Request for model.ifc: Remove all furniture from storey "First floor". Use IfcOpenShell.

First a look at what the model holds.

```python
import ifcopenshell
import ifcopenshell.util.element

model = ifcopenshell.open("model.ifc")
print(model.schema)
storey = next(s for s in model.by_type("IfcBuildingStorey") if s.Name == "First floor")
furniture = [e for e in ifcopenshell.util.element.get_decomposition(storey) if e.is_a("IfcFurnishingElement")]
seen = {}
for e in furniture:
    element_type = ifcopenshell.util.element.get_type(e)
    name = element_type.Name if element_type not in (None, e) else None
    seen[name] = seen.get(name, 0) + 1
for name, count in sorted(seen.items(), key=str):
    print(count, "x", name)
```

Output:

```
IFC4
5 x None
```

```python
import ifcopenshell
import ifcopenshell.api.root
import ifcopenshell.util.element

model = ifcopenshell.open("model.ifc")

storey = next(s for s in model.by_type("IfcBuildingStorey") if s.Name == "First floor")
furniture = [e for e in ifcopenshell.util.element.get_decomposition(storey) if e.is_a("IfcFurnishingElement")]

for e in furniture:
    ifcopenshell.api.root.remove_product(model, product=e)
print(len(furniture), "removed")

model.write("model_updated.ifc")
```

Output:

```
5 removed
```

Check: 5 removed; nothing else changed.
